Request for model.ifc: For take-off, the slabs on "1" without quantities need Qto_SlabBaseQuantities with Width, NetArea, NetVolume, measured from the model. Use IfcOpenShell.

First a look at what the model holds.

```python
import ifcopenshell
import ifcopenshell.util.element
import ifcopenshell.util.unit

model = ifcopenshell.open("model.ifc")
print(model.schema)
for unit_type in ("LENGTHUNIT", "AREAUNIT", "VOLUMEUNIT"):
    print(unit_type, ifcopenshell.util.unit.calculate_unit_scale(model, unit_type))
storey = next(s for s in model.by_type("IfcBuildingStorey") if s.Name == "1")
slabs = [e for e in ifcopenshell.util.element.get_decomposition(storey) if e.is_a("IfcSlab")]
for e in sorted(slabs, key=lambda e: e.id()):
    print(e.id(), e.is_a(), e.Name, list(ifcopenshell.util.element.get_psets(e, qtos_only=True)), sep=" | ")
```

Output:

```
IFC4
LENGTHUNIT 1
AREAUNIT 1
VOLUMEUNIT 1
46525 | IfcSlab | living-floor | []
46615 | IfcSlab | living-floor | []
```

```python
import ifcopenshell
import ifcopenshell.api.pset
import ifcopenshell.geom
import ifcopenshell.util.element
import ifcopenshell.util.shape
import ifcopenshell.util.unit

model = ifcopenshell.open("model.ifc")
unit_scale = ifcopenshell.util.unit.calculate_unit_scale(model)
area_scale = ifcopenshell.util.unit.calculate_unit_scale(model, "AREAUNIT")
volume_scale = ifcopenshell.util.unit.calculate_unit_scale(model, "VOLUMEUNIT")
settings = ifcopenshell.geom.settings()

storey = next(s for s in model.by_type("IfcBuildingStorey") if s.Name == "1")
slabs = [e for e in ifcopenshell.util.element.get_decomposition(storey) if e.is_a("IfcSlab")]

for e in sorted(slabs, key=lambda e: e.id()):
    if ifcopenshell.util.element.get_psets(e, qtos_only=True, should_inherit=False):
        continue
    # Geometry comes back in metres, in the element's own axes.
    shape = ifcopenshell.geom.create_shape(settings, e)
    values = {
        "Width": ifcopenshell.util.shape.get_z(shape.geometry) / unit_scale,
        "NetArea": ifcopenshell.util.shape.get_footprint_area(shape.geometry) / area_scale,
        "NetVolume": ifcopenshell.util.shape.get_volume(shape.geometry) / volume_scale,
    }
    qto = ifcopenshell.api.pset.add_qto(model, product=e, name="Qto_SlabBaseQuantities")
    ifcopenshell.api.pset.edit_qto(model, qto=qto, properties=values)
    print(e.id(), {k: round(v, 3) for k, v in values.items()})

model.write("model_updated.ifc")
```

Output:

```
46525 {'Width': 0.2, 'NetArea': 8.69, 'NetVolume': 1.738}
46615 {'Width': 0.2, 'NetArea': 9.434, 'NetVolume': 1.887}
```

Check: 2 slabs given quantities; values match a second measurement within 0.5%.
